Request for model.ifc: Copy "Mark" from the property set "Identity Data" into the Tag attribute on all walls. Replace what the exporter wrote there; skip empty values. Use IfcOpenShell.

First a look at what the model holds.

```python
import ifcopenshell
import ifcopenshell.util.element

model = ifcopenshell.open("model.ifc")
print(model.schema)
walls = model.by_type("IfcWall")
print(len(walls), "walls")
for e in walls[:8]:
    source = ifcopenshell.util.element.get_pset(e, "Identity Data", "Mark")
    target = e.Tag
    print(e.id(), repr(source), repr(target), sep=" | ")
```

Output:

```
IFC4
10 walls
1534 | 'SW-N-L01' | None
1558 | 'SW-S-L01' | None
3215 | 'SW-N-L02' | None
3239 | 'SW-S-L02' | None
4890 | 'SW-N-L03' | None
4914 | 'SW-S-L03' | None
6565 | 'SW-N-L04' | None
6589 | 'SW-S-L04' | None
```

```python
import ifcopenshell
import ifcopenshell.util.element

model = ifcopenshell.open("model.ifc")

count = 0
for e in model.by_type("IfcWall"):
    value = ifcopenshell.util.element.get_pset(e, "Identity Data", "Mark")
    current = e.Tag
    if not value or not value.strip() or current == value:
        continue
    e.Tag = value
    count += 1

print(count, "walls updated")

model.write("model_updated.ifc")
```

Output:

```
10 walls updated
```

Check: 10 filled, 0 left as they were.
